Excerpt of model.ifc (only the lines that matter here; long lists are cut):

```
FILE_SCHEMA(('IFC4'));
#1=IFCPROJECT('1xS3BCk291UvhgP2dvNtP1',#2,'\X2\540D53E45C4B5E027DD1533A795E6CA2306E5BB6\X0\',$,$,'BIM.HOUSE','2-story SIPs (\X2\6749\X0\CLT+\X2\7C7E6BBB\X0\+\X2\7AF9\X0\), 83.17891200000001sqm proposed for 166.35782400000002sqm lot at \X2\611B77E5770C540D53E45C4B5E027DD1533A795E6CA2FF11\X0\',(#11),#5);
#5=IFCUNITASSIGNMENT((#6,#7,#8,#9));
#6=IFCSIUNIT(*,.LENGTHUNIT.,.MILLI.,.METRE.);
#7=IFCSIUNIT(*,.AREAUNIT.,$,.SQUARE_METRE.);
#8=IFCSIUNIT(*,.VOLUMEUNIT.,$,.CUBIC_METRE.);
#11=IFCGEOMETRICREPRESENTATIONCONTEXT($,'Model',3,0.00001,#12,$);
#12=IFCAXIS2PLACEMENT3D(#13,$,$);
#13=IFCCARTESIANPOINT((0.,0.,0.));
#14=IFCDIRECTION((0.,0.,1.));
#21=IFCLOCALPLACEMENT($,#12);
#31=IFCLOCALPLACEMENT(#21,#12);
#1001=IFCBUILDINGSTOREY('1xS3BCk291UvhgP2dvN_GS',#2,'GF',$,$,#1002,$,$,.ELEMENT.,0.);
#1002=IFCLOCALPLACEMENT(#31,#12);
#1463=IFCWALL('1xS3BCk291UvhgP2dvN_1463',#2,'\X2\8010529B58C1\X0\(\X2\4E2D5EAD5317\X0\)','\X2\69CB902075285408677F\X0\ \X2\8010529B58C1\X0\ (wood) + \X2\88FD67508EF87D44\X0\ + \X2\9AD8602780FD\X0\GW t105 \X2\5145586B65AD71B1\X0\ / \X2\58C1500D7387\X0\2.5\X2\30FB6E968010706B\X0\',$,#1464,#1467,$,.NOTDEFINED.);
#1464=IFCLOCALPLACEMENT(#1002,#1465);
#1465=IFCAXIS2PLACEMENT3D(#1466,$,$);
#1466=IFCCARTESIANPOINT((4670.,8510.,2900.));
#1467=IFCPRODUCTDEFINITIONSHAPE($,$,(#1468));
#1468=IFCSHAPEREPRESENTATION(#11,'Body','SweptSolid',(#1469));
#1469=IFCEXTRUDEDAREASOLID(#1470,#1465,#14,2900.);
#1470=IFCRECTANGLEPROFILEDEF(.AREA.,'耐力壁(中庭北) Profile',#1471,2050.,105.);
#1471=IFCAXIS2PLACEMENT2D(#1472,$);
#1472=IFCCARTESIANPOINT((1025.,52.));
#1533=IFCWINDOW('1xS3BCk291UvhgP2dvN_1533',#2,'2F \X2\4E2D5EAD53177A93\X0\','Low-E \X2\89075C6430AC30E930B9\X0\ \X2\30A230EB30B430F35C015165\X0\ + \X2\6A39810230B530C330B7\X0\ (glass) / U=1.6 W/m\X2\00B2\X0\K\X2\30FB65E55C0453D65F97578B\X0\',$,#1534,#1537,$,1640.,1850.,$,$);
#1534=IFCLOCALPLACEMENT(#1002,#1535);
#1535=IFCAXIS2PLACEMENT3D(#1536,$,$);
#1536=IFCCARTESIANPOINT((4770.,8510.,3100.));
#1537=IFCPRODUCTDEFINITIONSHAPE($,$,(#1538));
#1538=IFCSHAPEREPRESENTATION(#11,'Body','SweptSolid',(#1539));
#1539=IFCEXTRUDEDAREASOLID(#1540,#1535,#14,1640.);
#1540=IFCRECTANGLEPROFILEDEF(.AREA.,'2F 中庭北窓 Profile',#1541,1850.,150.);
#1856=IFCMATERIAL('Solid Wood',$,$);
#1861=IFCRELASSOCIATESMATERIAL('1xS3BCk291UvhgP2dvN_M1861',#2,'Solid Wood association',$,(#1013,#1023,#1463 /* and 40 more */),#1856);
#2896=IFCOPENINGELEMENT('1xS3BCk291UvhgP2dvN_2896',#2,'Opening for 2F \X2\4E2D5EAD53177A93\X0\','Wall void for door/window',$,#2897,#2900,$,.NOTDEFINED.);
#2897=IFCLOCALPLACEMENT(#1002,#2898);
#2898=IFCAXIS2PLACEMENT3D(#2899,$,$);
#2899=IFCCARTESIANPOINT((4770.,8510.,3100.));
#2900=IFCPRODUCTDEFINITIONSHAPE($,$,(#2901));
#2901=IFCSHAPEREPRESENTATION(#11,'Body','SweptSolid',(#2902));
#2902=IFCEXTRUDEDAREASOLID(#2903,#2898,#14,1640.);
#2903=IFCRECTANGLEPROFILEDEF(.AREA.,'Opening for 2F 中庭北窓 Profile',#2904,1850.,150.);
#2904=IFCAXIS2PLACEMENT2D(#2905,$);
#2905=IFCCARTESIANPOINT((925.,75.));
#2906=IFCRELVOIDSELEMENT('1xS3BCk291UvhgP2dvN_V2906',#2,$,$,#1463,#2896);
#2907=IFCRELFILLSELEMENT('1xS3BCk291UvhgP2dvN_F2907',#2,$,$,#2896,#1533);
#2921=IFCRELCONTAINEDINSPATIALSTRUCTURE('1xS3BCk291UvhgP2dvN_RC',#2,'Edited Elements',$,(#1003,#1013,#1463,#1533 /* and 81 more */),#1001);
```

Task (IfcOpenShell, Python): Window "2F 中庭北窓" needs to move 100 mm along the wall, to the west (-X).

```python
import ifcopenshell
import ifcopenshell.api.geometry
import ifcopenshell.util.placement
import ifcopenshell.util.unit

model = ifcopenshell.open("model.ifc")
unit_scale = ifcopenshell.util.unit.calculate_unit_scale(model)

window = model.by_guid("1xS3BCk291UvhgP2dvN_1533")
opening = window.FillsVoids[0].RelatingOpeningElement
wall = opening.VoidsElements[0].RelatingBuildingElement

wall_matrix = ifcopenshell.util.placement.get_local_placement(wall.ObjectPlacement)
shift = wall_matrix[:3, 0] * -0.1 / unit_scale
before = ifcopenshell.util.placement.get_local_placement(window.ObjectPlacement)[:3, 3].copy()

# The window is not placed relative to its opening, so move both.
for product in (opening, window):
    matrix = ifcopenshell.util.placement.get_local_placement(product.ObjectPlacement)
    matrix[:3, 3] += shift
    ifcopenshell.api.geometry.edit_object_placement(model, product=product, matrix=matrix, is_si=False)

after = ifcopenshell.util.placement.get_local_placement(window.ObjectPlacement)[:3, 3]
print("window moved by", (after - before).round(3) + 0.0)

model.write("model_edited.ifc")
```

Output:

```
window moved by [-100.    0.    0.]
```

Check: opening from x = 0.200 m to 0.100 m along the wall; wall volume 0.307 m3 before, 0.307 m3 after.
